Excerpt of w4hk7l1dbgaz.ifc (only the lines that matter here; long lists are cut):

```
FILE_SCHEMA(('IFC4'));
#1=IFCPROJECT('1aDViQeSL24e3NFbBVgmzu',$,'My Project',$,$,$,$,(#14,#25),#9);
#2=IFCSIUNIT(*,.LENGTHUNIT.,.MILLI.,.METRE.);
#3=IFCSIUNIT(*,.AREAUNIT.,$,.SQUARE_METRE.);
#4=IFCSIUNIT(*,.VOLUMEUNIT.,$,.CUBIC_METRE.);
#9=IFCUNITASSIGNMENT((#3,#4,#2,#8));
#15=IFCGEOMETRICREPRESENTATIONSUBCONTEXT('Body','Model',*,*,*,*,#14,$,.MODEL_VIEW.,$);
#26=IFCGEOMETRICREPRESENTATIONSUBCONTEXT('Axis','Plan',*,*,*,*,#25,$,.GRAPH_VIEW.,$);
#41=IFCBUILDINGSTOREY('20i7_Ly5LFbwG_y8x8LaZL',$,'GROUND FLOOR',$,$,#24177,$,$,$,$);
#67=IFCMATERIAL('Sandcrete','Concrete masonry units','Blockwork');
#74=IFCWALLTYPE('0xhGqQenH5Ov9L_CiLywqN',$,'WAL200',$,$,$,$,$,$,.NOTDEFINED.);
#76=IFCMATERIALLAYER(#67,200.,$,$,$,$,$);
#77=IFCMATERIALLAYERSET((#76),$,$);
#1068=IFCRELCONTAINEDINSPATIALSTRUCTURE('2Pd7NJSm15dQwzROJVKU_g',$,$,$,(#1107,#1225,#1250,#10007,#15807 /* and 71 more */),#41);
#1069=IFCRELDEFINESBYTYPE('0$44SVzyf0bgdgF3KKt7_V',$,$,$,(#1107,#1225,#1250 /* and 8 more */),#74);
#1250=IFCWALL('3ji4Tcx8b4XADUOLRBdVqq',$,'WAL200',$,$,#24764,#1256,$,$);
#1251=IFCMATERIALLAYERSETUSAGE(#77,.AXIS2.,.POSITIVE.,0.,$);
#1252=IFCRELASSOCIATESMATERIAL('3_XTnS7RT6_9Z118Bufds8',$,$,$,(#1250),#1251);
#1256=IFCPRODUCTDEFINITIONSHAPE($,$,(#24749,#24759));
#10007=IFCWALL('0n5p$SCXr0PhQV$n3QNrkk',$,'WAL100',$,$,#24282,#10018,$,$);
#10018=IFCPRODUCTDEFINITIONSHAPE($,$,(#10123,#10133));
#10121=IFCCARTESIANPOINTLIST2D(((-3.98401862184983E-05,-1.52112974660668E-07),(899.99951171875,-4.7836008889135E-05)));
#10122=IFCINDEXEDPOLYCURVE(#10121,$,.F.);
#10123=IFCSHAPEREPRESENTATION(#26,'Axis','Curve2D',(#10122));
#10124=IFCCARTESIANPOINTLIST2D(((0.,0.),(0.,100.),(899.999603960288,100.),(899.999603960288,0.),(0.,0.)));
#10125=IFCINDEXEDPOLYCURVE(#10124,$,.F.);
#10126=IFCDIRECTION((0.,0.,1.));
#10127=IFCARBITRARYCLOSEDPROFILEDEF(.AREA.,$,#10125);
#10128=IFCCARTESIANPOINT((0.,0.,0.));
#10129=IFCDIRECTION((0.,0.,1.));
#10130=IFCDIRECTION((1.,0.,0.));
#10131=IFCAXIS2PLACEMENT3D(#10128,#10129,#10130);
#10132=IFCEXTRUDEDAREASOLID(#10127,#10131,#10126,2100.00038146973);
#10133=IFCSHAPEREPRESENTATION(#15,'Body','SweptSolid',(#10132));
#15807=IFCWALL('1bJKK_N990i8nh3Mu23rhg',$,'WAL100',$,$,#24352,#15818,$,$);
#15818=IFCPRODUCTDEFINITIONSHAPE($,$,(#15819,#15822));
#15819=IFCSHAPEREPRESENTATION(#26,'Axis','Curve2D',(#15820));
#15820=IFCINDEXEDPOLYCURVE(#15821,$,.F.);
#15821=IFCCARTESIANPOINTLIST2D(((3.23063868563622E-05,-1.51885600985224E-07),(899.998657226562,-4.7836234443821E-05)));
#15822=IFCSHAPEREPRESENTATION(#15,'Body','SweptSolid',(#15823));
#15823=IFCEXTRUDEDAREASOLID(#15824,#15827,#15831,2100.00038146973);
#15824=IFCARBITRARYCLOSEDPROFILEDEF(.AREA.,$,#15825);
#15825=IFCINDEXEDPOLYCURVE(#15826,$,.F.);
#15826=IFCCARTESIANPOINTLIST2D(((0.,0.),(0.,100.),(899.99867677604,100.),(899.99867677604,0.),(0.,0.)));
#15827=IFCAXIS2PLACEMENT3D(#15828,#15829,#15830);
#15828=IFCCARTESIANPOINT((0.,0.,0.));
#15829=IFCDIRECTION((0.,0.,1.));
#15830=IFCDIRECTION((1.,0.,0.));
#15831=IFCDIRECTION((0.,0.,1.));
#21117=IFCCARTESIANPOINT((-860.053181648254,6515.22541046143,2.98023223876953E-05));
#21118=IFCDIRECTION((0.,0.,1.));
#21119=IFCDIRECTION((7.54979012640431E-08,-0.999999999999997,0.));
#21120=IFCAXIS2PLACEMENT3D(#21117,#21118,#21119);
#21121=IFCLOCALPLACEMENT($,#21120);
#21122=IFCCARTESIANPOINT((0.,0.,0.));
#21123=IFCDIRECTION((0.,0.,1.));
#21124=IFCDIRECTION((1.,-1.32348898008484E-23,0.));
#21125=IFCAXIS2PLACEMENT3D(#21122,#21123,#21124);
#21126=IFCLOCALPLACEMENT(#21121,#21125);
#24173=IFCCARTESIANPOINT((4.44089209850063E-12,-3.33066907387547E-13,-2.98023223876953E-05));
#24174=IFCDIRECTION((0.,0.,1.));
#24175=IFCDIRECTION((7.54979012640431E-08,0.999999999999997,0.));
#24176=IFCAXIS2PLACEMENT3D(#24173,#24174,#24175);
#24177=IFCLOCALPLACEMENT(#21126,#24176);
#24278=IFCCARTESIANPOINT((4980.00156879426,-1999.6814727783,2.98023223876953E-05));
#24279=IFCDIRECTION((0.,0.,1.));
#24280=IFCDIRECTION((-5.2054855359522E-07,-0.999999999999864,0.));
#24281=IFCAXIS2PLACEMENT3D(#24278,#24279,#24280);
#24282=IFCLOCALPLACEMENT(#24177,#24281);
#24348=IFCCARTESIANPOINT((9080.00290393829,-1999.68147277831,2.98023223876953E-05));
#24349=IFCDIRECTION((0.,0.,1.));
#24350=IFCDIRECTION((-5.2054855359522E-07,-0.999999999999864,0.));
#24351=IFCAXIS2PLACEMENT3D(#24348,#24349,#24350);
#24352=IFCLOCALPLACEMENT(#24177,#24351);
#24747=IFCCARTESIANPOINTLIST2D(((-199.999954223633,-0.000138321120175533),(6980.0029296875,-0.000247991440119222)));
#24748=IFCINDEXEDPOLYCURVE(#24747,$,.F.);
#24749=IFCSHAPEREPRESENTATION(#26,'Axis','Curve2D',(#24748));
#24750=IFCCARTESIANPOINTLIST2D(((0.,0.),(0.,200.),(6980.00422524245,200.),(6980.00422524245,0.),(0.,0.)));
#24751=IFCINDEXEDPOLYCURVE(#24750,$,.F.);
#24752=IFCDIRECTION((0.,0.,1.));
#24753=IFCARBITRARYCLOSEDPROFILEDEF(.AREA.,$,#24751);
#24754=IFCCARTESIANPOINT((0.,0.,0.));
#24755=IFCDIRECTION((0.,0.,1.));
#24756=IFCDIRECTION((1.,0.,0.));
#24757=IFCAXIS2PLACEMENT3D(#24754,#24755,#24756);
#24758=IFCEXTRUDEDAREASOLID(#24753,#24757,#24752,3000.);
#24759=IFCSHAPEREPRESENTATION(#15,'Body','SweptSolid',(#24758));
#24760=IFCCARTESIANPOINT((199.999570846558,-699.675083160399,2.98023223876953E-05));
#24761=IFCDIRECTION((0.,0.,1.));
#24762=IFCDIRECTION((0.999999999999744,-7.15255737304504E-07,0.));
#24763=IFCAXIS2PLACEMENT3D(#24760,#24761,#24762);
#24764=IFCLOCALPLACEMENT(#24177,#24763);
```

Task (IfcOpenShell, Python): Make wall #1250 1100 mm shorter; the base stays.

```python
import ifcopenshell
import ifcopenshell.geom
import ifcopenshell.util.representation
import ifcopenshell.util.shape

model = ifcopenshell.open("w4hk7l1dbgaz.ifc")
settings = ifcopenshell.geom.settings()


def volume(element):
    """Net volume in cubic metres, openings subtracted."""
    shape = ifcopenshell.geom.create_shape(settings, element)
    return ifcopenshell.util.shape.get_volume(shape.geometry)


wall = model.by_guid("3ji4Tcx8b4XADUOLRBdVqq")
before = volume(wall)

body = ifcopenshell.util.representation.get_representation(wall, "Model", "Body")
solid = body.Items[0]
old_height = solid.Depth
solid.Depth -= 1100.0
after = volume(wall)

print(f"height {old_height:g} -> {solid.Depth:g}, volume {before:.3f} -> {after:.3f} m3")

model.write("w4hk7l1dbgaz_rev.ifc")
```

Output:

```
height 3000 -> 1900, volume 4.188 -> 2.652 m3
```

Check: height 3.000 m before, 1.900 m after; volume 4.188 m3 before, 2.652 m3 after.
